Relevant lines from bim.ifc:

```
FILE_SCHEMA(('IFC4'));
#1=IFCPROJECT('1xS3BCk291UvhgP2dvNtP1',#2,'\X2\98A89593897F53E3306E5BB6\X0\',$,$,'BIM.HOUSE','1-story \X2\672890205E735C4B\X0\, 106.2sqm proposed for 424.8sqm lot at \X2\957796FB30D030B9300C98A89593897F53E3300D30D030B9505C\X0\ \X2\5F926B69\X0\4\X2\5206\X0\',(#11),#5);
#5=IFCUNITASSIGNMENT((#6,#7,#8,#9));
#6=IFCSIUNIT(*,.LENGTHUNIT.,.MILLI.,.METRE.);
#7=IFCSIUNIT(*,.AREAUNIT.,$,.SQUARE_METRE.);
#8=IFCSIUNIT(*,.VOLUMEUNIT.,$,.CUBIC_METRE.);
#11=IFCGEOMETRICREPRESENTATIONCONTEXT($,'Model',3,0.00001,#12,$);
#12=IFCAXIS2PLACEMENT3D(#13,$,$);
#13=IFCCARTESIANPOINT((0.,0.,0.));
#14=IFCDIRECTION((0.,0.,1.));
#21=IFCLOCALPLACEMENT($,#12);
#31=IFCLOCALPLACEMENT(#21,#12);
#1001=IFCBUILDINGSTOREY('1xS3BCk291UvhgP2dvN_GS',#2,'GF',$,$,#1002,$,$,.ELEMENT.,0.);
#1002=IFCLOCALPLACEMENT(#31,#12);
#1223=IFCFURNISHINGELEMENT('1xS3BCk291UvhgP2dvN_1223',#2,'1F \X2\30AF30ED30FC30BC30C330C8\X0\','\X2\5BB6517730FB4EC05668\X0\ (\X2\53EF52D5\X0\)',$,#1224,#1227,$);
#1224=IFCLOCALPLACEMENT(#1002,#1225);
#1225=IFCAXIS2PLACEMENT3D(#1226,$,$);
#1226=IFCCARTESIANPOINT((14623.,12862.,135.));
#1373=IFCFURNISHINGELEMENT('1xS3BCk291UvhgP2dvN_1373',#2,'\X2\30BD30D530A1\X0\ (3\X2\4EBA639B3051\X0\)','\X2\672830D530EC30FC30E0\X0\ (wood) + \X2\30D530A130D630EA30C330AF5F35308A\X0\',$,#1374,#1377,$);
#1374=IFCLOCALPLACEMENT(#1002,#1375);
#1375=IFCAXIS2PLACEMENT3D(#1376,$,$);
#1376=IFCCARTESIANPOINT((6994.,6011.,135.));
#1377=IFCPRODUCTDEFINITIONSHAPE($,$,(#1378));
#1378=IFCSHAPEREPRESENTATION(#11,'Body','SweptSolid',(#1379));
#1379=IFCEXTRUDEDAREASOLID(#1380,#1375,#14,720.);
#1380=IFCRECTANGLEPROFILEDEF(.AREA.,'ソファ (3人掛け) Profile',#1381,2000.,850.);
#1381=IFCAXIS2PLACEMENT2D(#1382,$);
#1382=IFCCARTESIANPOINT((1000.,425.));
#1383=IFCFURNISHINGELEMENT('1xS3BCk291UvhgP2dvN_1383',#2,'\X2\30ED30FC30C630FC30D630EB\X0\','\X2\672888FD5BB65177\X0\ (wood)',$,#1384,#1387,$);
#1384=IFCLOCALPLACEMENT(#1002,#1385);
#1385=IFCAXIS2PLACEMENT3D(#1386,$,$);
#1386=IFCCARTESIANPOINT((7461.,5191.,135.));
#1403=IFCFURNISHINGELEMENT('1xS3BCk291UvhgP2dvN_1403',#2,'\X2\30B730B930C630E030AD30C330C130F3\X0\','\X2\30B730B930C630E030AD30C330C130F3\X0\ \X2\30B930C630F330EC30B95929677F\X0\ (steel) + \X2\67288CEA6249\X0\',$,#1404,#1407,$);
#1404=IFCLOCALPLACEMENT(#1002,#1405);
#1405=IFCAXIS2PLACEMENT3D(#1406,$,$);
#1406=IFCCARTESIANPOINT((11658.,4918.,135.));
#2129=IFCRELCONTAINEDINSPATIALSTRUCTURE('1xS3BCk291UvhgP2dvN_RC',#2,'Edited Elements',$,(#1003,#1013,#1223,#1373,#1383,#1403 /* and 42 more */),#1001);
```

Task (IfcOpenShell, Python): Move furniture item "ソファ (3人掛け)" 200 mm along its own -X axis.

```python
import ifcopenshell
import ifcopenshell.api.geometry
import ifcopenshell.util.placement
import ifcopenshell.util.unit

model = ifcopenshell.open("bim.ifc")
unit_scale = ifcopenshell.util.unit.calculate_unit_scale(model)

item = model.by_id(1373)
matrix = ifcopenshell.util.placement.get_local_placement(item.ObjectPlacement)
matrix[:3, 3] -= matrix[:3, 0] * 0.2 / unit_scale
ifcopenshell.api.geometry.edit_object_placement(model, product=item, matrix=matrix, is_si=False)

print(ifcopenshell.util.placement.get_local_placement(item.ObjectPlacement).round(3) + 0.0)

model.write("bim_updated.ifc")
```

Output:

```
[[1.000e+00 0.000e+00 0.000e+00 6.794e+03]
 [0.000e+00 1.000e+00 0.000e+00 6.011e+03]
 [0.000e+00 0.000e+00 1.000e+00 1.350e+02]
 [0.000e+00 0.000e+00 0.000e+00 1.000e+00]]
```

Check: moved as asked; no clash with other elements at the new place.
